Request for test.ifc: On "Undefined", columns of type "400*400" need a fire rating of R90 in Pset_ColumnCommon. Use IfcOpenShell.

First a look at what the model holds.

```python
import ifcopenshell
import ifcopenshell.util.element

model = ifcopenshell.open("test.ifc")
print(model.schema)
storey = next(s for s in model.by_type("IfcBuildingStorey") if s.Name == "Undefined")
columns = [e for e in ifcopenshell.util.element.get_decomposition(storey) if e.is_a("IfcColumn")]
seen = {}
for e in columns:
    element_type = ifcopenshell.util.element.get_type(e)
    key = (element_type.Name if element_type != e and element_type else None, ifcopenshell.util.element.get_pset(e, "Pset_ColumnCommon", "FireRating"))
    seen[key] = seen.get(key, 0) + 1
for (name, value), count in sorted(seen.items(), key=str):
    print(count, "x", name, "|", value)
```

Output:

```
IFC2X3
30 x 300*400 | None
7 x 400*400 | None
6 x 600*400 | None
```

```python
import ifcopenshell
import ifcopenshell.api.pset
import ifcopenshell.util.element

model = ifcopenshell.open("test.ifc")

storey = next(s for s in model.by_type("IfcBuildingStorey") if s.Name == "Undefined")
columns = [e for e in ifcopenshell.util.element.get_decomposition(storey) if e.is_a("IfcColumn")]

count = 0
for e in columns:
    element_type = ifcopenshell.util.element.get_type(e)
    if element_type in (None, e) or element_type.Name != "400*400":
        continue
    found = ifcopenshell.util.element.get_pset(e, "Pset_ColumnCommon", should_inherit=False)
    if found:
        pset = model.by_id(found["id"])
        if len(ifcopenshell.util.element.get_elements_by_pset(pset)) > 1:
            pset = ifcopenshell.api.pset.unshare_pset(model, products=[e], pset=pset)[0]
    else:
        pset = ifcopenshell.api.pset.add_pset(model, product=e, name="Pset_ColumnCommon")
    ifcopenshell.api.pset.edit_pset(model, pset=pset, properties={"FireRating": "R90"})
    count += 1

print(count, "columns updated")

model.write("test-out.ifc")
```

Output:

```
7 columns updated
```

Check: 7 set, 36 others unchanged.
